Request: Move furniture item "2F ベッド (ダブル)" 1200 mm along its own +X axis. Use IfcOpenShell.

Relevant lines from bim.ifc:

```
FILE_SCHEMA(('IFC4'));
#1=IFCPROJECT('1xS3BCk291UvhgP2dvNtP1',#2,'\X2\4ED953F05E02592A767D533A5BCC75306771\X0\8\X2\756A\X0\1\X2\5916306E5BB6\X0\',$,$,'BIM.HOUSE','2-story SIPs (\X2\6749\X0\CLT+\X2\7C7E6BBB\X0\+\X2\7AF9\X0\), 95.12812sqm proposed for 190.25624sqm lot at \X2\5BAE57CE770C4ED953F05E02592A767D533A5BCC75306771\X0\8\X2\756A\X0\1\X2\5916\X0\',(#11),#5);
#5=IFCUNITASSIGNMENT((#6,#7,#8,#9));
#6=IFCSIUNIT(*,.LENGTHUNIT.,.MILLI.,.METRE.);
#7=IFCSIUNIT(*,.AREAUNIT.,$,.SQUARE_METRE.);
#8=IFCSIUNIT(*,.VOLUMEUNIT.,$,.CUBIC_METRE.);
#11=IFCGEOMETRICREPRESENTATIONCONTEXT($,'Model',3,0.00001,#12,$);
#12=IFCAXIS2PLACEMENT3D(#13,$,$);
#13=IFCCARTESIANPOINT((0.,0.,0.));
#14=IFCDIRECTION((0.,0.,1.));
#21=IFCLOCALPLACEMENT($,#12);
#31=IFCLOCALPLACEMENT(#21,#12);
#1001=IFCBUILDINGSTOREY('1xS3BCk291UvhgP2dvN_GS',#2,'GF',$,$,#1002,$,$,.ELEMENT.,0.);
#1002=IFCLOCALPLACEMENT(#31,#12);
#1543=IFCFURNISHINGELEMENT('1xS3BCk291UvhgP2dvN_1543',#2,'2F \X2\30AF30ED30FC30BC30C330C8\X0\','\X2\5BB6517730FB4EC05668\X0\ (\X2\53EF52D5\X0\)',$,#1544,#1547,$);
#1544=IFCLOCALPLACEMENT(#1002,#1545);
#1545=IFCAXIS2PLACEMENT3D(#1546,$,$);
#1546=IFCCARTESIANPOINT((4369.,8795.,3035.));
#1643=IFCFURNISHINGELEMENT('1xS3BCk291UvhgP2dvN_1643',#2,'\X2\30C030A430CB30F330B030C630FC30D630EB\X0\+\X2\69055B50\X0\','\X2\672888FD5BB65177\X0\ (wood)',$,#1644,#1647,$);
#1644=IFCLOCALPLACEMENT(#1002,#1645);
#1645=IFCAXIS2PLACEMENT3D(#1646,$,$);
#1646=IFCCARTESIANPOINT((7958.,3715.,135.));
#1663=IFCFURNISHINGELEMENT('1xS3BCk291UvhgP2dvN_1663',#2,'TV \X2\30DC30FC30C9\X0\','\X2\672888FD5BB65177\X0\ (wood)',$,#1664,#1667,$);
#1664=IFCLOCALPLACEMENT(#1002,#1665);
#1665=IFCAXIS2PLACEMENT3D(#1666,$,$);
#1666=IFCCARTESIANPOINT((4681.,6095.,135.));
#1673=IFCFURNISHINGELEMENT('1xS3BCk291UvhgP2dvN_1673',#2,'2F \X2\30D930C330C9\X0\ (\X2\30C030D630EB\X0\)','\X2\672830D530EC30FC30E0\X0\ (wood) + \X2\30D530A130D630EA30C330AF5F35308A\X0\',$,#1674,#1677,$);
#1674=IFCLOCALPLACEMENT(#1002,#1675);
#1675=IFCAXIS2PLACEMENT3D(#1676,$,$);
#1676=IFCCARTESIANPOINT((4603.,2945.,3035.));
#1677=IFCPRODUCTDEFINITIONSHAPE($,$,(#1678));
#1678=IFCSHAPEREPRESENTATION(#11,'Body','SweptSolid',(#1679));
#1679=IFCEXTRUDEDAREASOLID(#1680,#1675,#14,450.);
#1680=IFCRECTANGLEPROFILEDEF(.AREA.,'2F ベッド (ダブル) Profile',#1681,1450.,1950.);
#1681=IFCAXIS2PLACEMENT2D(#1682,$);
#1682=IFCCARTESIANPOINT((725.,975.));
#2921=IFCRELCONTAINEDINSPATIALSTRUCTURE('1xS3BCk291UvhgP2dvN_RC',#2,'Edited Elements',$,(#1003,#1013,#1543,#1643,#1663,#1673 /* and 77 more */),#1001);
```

```python
import ifcopenshell
import ifcopenshell.api.geometry
import ifcopenshell.util.placement

model = ifcopenshell.open("bim.ifc")

item = model.by_guid("1xS3BCk291UvhgP2dvN_1673")
matrix = ifcopenshell.util.placement.get_local_placement(item.ObjectPlacement)
matrix[:3, 3] += matrix[:3, 0] * 1200.0
ifcopenshell.api.geometry.edit_object_placement(model, product=item, matrix=matrix, is_si=False)

print(ifcopenshell.util.placement.get_local_placement(item.ObjectPlacement).round(3) + 0.0)

model.write("bim_rev.ifc")
```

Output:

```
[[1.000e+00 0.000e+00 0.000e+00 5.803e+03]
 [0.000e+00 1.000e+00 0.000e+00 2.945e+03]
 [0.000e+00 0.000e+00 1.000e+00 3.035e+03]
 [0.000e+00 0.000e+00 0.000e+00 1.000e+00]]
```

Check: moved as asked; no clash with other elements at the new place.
